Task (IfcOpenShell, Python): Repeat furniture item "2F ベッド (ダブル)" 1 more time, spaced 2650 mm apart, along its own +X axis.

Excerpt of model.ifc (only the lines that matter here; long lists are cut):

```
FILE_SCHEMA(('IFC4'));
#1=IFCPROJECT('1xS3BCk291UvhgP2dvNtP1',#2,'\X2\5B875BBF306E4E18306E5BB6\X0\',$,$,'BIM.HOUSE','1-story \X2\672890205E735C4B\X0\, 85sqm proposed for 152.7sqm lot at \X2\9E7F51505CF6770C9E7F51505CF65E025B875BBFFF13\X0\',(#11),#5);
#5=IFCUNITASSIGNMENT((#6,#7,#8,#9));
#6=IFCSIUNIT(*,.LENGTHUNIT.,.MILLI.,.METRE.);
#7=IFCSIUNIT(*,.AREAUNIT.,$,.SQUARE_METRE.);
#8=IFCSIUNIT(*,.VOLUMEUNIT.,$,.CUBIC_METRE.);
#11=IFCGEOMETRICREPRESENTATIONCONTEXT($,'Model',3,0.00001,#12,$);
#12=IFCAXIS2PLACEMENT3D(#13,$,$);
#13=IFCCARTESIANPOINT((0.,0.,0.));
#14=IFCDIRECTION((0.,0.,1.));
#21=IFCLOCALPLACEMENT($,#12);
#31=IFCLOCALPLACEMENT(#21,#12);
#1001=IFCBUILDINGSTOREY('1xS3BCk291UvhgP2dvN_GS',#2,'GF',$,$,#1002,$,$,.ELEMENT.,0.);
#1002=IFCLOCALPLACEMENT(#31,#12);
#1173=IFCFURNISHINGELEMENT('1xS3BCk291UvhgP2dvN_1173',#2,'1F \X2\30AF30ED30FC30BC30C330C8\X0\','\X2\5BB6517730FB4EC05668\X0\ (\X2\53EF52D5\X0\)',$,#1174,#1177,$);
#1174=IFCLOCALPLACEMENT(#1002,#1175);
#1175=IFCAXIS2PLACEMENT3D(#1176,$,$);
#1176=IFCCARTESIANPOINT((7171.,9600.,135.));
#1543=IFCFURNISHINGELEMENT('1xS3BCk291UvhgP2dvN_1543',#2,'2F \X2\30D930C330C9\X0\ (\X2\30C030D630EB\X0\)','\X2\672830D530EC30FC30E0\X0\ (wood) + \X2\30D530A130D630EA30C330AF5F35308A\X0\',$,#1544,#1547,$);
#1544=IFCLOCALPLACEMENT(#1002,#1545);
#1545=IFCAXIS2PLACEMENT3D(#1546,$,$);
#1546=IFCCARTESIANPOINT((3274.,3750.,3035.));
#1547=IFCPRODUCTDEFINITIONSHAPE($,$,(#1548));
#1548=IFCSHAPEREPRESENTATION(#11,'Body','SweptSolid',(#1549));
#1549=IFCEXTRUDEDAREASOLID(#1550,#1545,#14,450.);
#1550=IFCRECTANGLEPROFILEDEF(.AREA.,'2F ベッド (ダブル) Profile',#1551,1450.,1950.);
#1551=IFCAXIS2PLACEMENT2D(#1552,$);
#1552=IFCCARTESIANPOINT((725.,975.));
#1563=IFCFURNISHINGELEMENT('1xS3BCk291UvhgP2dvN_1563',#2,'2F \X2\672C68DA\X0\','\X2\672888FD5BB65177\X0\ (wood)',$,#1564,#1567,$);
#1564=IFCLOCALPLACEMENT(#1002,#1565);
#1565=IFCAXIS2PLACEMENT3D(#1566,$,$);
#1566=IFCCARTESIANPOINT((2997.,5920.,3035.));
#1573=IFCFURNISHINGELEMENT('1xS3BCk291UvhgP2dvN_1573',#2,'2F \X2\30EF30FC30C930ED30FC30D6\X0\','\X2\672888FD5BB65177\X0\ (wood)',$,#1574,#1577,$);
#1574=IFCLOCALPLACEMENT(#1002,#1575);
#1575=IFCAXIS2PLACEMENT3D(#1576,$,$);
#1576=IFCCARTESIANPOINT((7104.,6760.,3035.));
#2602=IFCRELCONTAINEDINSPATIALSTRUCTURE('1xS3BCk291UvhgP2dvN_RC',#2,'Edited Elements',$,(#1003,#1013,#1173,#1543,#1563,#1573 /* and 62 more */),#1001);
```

```python
import ifcopenshell
import ifcopenshell.api.geometry
import ifcopenshell.api.root
import ifcopenshell.util.element
import ifcopenshell.util.placement
import ifcopenshell.util.unit

model = ifcopenshell.open("model.ifc")
unit_scale = ifcopenshell.util.unit.calculate_unit_scale(model)


def reuse_history(source, copy):
    """copy_class also copies each property set's owner history, people and application; keep the originals."""
    for rel in copy.IsDefinedBy:
        if rel.is_a("IfcRelDefinesByProperties") and (history := rel.RelatingPropertyDefinition.OwnerHistory):
            rel.RelatingPropertyDefinition.OwnerHistory = source.OwnerHistory
            ifcopenshell.util.element.remove_deep2(model, history)


source = model.by_guid("1xS3BCk291UvhgP2dvN_1543")
base = ifcopenshell.util.placement.get_local_placement(source.ObjectPlacement)
step = base[:3, 0] * 2.65 / unit_scale

for i in range(1, 2):
    copy = ifcopenshell.api.root.copy_class(model, product=source)
    copy.Representation = ifcopenshell.util.element.copy_deep(
        model, source.Representation, exclude=["IfcGeometricRepresentationContext", "IfcRepresentationMap"]
    )
    reuse_history(source, copy)
    matrix = base.copy()
    matrix[:3, 3] += i * step
    print("added at", matrix[:3, 3].round(3) + 0.0)
    ifcopenshell.api.geometry.edit_object_placement(model, product=copy, matrix=matrix, is_si=False)

model.write("model_rev.ifc")
```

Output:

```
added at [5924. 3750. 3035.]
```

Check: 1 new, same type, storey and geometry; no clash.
